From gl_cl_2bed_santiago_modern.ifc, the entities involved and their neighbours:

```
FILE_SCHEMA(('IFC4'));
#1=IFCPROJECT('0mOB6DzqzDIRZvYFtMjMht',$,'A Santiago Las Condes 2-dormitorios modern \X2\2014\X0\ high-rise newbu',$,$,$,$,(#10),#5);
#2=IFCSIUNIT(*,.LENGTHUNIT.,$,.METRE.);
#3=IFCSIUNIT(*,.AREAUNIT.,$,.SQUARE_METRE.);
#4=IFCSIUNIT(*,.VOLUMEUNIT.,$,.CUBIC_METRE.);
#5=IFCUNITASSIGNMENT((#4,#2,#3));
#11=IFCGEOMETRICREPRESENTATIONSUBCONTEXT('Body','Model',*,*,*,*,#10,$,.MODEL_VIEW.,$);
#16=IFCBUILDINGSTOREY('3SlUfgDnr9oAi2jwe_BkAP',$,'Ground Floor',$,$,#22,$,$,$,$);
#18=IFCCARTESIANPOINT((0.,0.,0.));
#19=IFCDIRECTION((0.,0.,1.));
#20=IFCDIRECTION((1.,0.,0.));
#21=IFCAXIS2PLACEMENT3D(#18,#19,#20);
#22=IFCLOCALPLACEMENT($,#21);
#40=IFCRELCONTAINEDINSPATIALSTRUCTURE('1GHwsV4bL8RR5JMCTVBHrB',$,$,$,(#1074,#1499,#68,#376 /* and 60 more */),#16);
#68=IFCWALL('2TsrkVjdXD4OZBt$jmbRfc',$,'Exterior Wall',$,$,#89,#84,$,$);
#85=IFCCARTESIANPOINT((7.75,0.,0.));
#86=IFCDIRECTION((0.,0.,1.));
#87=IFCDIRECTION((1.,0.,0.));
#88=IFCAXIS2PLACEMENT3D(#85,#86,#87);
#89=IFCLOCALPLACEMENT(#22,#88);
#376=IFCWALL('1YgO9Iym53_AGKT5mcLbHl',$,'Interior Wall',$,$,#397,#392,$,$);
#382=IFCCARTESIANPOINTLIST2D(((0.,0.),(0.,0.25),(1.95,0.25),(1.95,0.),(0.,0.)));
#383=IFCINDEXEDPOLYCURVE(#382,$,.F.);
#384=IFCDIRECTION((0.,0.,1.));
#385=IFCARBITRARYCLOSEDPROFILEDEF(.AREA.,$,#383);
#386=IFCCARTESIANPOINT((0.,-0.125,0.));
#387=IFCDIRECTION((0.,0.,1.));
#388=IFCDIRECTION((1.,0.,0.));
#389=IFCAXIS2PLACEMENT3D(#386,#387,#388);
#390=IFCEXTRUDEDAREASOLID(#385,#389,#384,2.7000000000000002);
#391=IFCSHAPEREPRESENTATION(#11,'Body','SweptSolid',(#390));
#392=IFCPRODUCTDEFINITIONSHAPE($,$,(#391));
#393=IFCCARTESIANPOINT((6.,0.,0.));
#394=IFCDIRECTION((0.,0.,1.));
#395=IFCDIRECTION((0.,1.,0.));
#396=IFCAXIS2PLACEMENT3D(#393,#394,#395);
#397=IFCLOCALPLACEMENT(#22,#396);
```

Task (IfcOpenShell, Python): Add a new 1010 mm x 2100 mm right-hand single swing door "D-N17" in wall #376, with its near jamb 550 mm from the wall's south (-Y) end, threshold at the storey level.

```python
import numpy as np
import ifcopenshell
import ifcopenshell.api.feature
import ifcopenshell.api.geometry
import ifcopenshell.api.root
import ifcopenshell.api.spatial
import ifcopenshell.geom
import ifcopenshell.util.element
import ifcopenshell.util.placement
import ifcopenshell.util.representation
import ifcopenshell.util.shape
import ifcopenshell.util.unit

model = ifcopenshell.open("gl_cl_2bed_santiago_modern.ifc")
unit_scale = ifcopenshell.util.unit.calculate_unit_scale(model)
settings = ifcopenshell.geom.settings()


def volume(element):
    """Net volume in cubic metres, openings subtracted."""
    shape = ifcopenshell.geom.create_shape(settings, element)
    return ifcopenshell.util.shape.get_volume(shape.geometry)


wall = model.by_guid("1YgO9Iym53_AGKT5mcLbHl")
storey = ifcopenshell.util.element.get_container(wall, ifc_class="IfcBuildingStorey")
context = ifcopenshell.util.representation.get_context(model, "Model", "Body", "MODEL_VIEW")
before = volume(wall)

width, height, from_end, sill = 1.01, 2.1, 0.55, 0.0  # metres

# The wall runs along its own X axis, and the end named is its -X end.
wall_shape = ifcopenshell.geom.create_shape(settings, wall)
x, y, z = ifcopenshell.util.shape.get_vertices(wall_shape.geometry).T
start = x.min() + from_end
face, thickness = float(y.min()), float(y.max() - y.min())
wall_matrix = ifcopenshell.util.placement.get_local_placement(wall.ObjectPlacement)
level = ifcopenshell.util.placement.get_local_placement(storey.ObjectPlacement)[2, 3]


def in_wall(x, y):
    """Placement at x, y metres in the wall's axes, at sill height."""
    matrix = wall_matrix.copy()
    matrix[:, 3] = wall_matrix @ np.array([x / unit_scale, y / unit_scale, 0.0, 1.0])
    matrix[2, 3] = level + sill / unit_scale
    return matrix


# Opening: a box that overshoots both wall faces by 50 mm.
opening = ifcopenshell.api.root.create_entity(model, ifc_class="IfcOpeningElement", predefined_type="OPENING")
box = ifcopenshell.api.geometry.add_wall_representation(
    model, context=context, length=width, height=height, thickness=thickness + 0.1
)
ifcopenshell.api.geometry.assign_representation(model, product=opening, representation=box)
ifcopenshell.api.geometry.edit_object_placement(model, product=opening, matrix=in_wall(start, face - 0.05), is_si=False)
ifcopenshell.api.feature.add_feature(model, feature=opening, element=wall)

door = ifcopenshell.api.root.create_entity(model, ifc_class="IfcDoor", name="D-N17", predefined_type="DOOR")
door.OverallWidth, door.OverallHeight = width / unit_scale, height / unit_scale
door.OperationType = "SINGLE_SWING_RIGHT"
body = ifcopenshell.api.geometry.add_door_representation(
    model,
    context=context,
    overall_width=door.OverallWidth,
    overall_height=door.OverallHeight,
    operation_type="SINGLE_SWING_RIGHT",
    lining_properties={"LiningDepth": thickness / unit_scale, "ThresholdDepth": thickness / unit_scale},
)
ifcopenshell.api.geometry.assign_representation(model, product=door, representation=body)
ifcopenshell.api.spatial.assign_container(model, products=[door], relating_structure=storey)
ifcopenshell.api.feature.add_filling(model, opening=opening, element=door)

# The lining spans the wall, so the door starts at the wall face.
ifcopenshell.api.geometry.edit_object_placement(model, product=door, matrix=in_wall(start, face), is_si=False)

after = volume(wall)

print(f"wall volume {before:.3f} -> {after:.3f} m3")

model.write("gl_cl_2bed_santiago_modern-out.ifc")
```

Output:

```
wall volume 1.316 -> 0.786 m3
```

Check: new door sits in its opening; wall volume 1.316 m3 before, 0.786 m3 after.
